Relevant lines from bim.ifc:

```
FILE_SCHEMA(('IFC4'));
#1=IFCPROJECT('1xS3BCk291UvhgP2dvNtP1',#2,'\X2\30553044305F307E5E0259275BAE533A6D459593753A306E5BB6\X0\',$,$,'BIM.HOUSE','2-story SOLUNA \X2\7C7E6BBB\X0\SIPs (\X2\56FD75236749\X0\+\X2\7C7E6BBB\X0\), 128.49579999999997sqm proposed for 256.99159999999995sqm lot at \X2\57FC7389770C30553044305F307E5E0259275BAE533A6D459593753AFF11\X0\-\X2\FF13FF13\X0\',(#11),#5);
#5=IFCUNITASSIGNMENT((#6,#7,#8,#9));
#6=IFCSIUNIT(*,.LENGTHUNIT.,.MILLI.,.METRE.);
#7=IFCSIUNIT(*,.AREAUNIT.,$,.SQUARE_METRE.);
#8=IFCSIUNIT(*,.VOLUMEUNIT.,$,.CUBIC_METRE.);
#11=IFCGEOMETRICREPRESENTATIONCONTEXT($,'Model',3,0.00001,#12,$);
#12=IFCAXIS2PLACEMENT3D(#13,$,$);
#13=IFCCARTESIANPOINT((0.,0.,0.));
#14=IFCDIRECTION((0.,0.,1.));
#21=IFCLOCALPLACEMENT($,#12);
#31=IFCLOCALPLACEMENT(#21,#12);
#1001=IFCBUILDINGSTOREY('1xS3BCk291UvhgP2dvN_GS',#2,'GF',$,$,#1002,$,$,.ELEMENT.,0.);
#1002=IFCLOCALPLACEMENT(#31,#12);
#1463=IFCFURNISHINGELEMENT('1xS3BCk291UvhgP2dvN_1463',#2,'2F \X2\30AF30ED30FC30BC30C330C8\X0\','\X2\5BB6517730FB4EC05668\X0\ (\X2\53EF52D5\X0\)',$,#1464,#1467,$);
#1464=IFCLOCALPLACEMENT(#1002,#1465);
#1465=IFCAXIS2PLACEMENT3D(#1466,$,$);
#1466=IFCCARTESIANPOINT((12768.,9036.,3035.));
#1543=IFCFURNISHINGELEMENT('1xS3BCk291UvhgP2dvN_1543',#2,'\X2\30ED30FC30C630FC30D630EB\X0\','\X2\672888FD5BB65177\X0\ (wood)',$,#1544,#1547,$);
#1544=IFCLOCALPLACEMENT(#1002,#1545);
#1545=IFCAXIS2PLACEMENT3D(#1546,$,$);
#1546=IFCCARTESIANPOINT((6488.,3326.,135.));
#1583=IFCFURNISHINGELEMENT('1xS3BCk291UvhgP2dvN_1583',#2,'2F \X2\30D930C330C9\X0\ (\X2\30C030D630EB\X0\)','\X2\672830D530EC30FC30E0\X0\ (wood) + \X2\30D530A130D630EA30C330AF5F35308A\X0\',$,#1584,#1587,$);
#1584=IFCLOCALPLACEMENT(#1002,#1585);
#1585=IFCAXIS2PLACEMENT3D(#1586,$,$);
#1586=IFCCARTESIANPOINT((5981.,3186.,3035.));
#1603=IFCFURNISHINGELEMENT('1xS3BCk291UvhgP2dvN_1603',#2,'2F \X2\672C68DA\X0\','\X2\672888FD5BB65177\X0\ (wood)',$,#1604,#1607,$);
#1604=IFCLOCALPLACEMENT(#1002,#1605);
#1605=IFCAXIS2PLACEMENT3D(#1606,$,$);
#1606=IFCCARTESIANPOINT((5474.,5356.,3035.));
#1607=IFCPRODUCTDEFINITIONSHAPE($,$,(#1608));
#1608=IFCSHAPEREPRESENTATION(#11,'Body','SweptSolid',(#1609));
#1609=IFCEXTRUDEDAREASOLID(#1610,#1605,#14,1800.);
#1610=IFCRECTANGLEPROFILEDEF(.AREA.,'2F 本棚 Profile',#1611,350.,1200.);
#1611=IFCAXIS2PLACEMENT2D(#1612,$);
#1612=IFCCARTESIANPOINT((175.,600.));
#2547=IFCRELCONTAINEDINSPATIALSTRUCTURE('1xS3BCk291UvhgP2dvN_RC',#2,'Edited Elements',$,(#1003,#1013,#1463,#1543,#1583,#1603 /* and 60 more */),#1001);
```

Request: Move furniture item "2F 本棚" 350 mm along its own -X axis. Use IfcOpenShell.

```python
import ifcopenshell
import ifcopenshell.api.geometry
import ifcopenshell.util.placement
import ifcopenshell.util.unit

model = ifcopenshell.open("bim.ifc")
unit_scale = ifcopenshell.util.unit.calculate_unit_scale(model)

item = model.by_id(1603)
matrix = ifcopenshell.util.placement.get_local_placement(item.ObjectPlacement)
matrix[:3, 3] -= matrix[:3, 0] * 0.35 / unit_scale
ifcopenshell.api.geometry.edit_object_placement(model, product=item, matrix=matrix, is_si=False)

print(ifcopenshell.util.placement.get_local_placement(item.ObjectPlacement).round(3) + 0.0)

model.write("bim_v2.ifc")
```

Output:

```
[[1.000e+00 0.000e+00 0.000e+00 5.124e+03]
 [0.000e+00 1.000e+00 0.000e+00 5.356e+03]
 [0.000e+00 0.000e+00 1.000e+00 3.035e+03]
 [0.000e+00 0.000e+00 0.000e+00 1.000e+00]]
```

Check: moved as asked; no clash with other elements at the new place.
